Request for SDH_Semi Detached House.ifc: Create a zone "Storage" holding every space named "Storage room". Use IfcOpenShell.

First a look at what the model holds.

```python
import ifcopenshell

model = ifcopenshell.open("SDH_Semi Detached House.ifc")
print(model.schema)
seen = {}
for space in model.by_type("IfcSpace"):
    seen[space.LongName] = seen.get(space.LongName, 0) + 1
for name, count in sorted(seen.items(), key=str):
    print(count, "x", name)
print("zones:", [z.Name for z in model.by_type("IfcZone")][:20])
```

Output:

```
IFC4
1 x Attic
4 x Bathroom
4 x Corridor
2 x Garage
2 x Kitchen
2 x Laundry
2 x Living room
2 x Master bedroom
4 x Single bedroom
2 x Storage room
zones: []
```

```python
import ifcopenshell
import ifcopenshell.api.group
import ifcopenshell.api.root

model = ifcopenshell.open("SDH_Semi Detached House.ifc")

names = {"Storage room"}
spaces = [s for s in model.by_type("IfcSpace") if s.LongName in names]

zone = ifcopenshell.api.root.create_entity(model, ifc_class="IfcZone", name="Storage")
ifcopenshell.api.group.assign_group(model, products=spaces, group=zone)
print(len(spaces), "spaces in", zone.Name)

model.write("SDH_Semi Detached House_edited.ifc")
```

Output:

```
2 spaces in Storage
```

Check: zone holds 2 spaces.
